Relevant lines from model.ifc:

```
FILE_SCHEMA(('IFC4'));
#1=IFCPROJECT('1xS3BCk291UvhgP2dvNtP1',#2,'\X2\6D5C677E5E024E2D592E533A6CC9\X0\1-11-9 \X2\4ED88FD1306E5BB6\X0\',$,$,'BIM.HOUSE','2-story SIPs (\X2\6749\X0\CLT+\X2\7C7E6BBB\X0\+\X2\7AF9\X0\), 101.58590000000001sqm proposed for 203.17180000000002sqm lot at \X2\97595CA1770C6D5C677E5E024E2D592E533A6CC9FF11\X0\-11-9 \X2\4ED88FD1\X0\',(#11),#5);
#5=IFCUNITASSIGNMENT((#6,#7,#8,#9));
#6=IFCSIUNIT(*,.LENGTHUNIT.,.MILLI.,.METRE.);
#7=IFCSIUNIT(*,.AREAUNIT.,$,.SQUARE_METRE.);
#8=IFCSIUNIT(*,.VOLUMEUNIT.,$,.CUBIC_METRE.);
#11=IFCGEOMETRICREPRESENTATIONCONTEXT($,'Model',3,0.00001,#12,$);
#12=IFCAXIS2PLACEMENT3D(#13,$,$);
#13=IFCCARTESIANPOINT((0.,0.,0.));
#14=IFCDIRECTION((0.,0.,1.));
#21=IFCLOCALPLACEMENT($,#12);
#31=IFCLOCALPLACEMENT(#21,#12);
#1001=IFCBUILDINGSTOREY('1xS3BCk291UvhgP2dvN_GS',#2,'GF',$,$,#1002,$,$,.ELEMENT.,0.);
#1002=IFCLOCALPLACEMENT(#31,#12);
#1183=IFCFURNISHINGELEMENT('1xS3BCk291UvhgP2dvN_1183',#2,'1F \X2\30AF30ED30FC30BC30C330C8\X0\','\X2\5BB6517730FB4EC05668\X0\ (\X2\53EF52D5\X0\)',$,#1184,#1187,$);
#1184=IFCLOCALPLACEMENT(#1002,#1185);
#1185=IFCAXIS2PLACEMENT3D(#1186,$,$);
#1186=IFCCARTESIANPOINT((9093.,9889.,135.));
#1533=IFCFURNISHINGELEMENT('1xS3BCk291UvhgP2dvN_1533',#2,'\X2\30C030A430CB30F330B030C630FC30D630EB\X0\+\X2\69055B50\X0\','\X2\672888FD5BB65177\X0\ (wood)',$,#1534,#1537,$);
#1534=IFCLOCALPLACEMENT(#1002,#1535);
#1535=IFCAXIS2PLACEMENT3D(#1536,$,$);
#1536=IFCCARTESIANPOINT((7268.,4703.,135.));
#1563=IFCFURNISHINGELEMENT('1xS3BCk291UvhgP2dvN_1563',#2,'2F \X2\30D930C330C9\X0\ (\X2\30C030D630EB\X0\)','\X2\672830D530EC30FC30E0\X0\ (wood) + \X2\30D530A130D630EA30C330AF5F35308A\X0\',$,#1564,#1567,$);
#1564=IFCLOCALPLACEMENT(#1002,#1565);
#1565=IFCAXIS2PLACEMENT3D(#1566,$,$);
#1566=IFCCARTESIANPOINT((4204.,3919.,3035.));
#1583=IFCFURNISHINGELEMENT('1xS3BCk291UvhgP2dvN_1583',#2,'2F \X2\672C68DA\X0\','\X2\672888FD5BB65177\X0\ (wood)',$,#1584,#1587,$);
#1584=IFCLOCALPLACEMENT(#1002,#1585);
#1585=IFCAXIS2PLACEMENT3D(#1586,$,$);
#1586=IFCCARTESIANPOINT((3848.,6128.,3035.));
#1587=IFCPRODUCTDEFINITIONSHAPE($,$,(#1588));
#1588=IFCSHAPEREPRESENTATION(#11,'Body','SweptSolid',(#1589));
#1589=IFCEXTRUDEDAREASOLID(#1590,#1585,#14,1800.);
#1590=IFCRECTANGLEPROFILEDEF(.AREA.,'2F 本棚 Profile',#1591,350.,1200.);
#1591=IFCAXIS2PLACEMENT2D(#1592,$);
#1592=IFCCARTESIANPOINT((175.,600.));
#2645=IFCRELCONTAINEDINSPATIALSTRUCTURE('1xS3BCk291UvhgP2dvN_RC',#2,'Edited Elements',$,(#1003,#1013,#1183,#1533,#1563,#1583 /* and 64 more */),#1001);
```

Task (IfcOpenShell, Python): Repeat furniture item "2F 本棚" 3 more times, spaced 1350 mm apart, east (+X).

```python
import numpy as np
import ifcopenshell
import ifcopenshell.api.geometry
import ifcopenshell.api.root
import ifcopenshell.util.element
import ifcopenshell.util.placement

model = ifcopenshell.open("model.ifc")


def reuse_history(source, copy):
    """copy_class also copies each property set's owner history, people and application; keep the originals."""
    for rel in copy.IsDefinedBy:
        if rel.is_a("IfcRelDefinesByProperties") and (history := rel.RelatingPropertyDefinition.OwnerHistory):
            rel.RelatingPropertyDefinition.OwnerHistory = source.OwnerHistory
            ifcopenshell.util.element.remove_deep2(model, history)


source = model.by_guid("1xS3BCk291UvhgP2dvN_1583")
base = ifcopenshell.util.placement.get_local_placement(source.ObjectPlacement)
step = np.array([1.0, 0.0, 0.0]) * 1350.0

for i in range(1, 4):
    copy = ifcopenshell.api.root.copy_class(model, product=source)
    copy.Representation = ifcopenshell.util.element.copy_deep(
        model, source.Representation, exclude=["IfcGeometricRepresentationContext", "IfcRepresentationMap"]
    )
    reuse_history(source, copy)
    matrix = base.copy()
    matrix[:3, 3] += i * step
    print("added at", matrix[:3, 3].round(3) + 0.0)
    ifcopenshell.api.geometry.edit_object_placement(model, product=copy, matrix=matrix, is_si=False)

model.write("model_rev.ifc")
```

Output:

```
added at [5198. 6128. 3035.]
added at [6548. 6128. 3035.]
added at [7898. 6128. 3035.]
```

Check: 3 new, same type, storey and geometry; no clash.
